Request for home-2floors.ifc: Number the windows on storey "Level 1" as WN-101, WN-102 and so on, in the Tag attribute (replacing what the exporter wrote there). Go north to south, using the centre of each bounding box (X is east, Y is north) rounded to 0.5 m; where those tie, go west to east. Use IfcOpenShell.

First a look at what the model holds.

```python
import ifcopenshell
import ifcopenshell.util.element
import ifcopenshell.util.placement

model = ifcopenshell.open("home-2floors.ifc")
print(model.schema)
storey = next(s for s in model.by_type("IfcBuildingStorey") if s.Name == "Level 1")
windows = [e for e in ifcopenshell.util.element.get_decomposition(storey) if e.is_a("IfcWindow")]
for e in sorted(windows, key=lambda e: e.id()):
    origin = ifcopenshell.util.placement.get_local_placement(e.ObjectPlacement)[:3, 3]
    print(e.id(), e.Tag, e.Name, origin.round(2) + 0.0, sep=" | ")
```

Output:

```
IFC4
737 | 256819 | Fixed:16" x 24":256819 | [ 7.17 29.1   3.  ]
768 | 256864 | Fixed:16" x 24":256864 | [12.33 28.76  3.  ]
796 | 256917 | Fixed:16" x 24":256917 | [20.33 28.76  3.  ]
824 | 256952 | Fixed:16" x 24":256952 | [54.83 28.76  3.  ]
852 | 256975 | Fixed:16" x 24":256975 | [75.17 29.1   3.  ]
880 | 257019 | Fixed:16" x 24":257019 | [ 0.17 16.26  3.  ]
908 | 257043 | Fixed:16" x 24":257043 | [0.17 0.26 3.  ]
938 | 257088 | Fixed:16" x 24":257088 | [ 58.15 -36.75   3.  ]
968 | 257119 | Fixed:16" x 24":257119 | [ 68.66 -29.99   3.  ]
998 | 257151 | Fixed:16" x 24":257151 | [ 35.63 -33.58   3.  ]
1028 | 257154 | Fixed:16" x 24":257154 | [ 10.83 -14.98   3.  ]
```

```python
import ifcopenshell
import ifcopenshell.geom
import ifcopenshell.util.element
import ifcopenshell.util.shape

model = ifcopenshell.open("home-2floors.ifc")
settings = ifcopenshell.geom.settings()
settings.set("use-world-coords", True)


def centre(element):
    shape = ifcopenshell.geom.create_shape(settings, element)
    return ifcopenshell.util.shape.get_bbox_centroid(shape.geometry)


storey = next(s for s in model.by_type("IfcBuildingStorey") if s.Name == "Level 1")
windows = [e for e in ifcopenshell.util.element.get_decomposition(storey) if e.is_a("IfcWindow")]

# Insertion points can sit at a corner or the storey origin, so sort by the geometry (in metres).
centres = {e: centre(e) for e in windows}
windows.sort(key=lambda e: (-round(centres[e][1] / 0.5), centres[e][0]))

for i, e in enumerate(windows, start=1):
    number = f"WN-1{i:02d}"
    e.Tag = number
    print(e.id(), number)

model.write("home-2floors-out.ifc")
```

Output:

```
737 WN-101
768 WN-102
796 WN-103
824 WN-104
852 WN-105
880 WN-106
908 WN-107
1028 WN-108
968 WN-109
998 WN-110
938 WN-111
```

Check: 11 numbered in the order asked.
